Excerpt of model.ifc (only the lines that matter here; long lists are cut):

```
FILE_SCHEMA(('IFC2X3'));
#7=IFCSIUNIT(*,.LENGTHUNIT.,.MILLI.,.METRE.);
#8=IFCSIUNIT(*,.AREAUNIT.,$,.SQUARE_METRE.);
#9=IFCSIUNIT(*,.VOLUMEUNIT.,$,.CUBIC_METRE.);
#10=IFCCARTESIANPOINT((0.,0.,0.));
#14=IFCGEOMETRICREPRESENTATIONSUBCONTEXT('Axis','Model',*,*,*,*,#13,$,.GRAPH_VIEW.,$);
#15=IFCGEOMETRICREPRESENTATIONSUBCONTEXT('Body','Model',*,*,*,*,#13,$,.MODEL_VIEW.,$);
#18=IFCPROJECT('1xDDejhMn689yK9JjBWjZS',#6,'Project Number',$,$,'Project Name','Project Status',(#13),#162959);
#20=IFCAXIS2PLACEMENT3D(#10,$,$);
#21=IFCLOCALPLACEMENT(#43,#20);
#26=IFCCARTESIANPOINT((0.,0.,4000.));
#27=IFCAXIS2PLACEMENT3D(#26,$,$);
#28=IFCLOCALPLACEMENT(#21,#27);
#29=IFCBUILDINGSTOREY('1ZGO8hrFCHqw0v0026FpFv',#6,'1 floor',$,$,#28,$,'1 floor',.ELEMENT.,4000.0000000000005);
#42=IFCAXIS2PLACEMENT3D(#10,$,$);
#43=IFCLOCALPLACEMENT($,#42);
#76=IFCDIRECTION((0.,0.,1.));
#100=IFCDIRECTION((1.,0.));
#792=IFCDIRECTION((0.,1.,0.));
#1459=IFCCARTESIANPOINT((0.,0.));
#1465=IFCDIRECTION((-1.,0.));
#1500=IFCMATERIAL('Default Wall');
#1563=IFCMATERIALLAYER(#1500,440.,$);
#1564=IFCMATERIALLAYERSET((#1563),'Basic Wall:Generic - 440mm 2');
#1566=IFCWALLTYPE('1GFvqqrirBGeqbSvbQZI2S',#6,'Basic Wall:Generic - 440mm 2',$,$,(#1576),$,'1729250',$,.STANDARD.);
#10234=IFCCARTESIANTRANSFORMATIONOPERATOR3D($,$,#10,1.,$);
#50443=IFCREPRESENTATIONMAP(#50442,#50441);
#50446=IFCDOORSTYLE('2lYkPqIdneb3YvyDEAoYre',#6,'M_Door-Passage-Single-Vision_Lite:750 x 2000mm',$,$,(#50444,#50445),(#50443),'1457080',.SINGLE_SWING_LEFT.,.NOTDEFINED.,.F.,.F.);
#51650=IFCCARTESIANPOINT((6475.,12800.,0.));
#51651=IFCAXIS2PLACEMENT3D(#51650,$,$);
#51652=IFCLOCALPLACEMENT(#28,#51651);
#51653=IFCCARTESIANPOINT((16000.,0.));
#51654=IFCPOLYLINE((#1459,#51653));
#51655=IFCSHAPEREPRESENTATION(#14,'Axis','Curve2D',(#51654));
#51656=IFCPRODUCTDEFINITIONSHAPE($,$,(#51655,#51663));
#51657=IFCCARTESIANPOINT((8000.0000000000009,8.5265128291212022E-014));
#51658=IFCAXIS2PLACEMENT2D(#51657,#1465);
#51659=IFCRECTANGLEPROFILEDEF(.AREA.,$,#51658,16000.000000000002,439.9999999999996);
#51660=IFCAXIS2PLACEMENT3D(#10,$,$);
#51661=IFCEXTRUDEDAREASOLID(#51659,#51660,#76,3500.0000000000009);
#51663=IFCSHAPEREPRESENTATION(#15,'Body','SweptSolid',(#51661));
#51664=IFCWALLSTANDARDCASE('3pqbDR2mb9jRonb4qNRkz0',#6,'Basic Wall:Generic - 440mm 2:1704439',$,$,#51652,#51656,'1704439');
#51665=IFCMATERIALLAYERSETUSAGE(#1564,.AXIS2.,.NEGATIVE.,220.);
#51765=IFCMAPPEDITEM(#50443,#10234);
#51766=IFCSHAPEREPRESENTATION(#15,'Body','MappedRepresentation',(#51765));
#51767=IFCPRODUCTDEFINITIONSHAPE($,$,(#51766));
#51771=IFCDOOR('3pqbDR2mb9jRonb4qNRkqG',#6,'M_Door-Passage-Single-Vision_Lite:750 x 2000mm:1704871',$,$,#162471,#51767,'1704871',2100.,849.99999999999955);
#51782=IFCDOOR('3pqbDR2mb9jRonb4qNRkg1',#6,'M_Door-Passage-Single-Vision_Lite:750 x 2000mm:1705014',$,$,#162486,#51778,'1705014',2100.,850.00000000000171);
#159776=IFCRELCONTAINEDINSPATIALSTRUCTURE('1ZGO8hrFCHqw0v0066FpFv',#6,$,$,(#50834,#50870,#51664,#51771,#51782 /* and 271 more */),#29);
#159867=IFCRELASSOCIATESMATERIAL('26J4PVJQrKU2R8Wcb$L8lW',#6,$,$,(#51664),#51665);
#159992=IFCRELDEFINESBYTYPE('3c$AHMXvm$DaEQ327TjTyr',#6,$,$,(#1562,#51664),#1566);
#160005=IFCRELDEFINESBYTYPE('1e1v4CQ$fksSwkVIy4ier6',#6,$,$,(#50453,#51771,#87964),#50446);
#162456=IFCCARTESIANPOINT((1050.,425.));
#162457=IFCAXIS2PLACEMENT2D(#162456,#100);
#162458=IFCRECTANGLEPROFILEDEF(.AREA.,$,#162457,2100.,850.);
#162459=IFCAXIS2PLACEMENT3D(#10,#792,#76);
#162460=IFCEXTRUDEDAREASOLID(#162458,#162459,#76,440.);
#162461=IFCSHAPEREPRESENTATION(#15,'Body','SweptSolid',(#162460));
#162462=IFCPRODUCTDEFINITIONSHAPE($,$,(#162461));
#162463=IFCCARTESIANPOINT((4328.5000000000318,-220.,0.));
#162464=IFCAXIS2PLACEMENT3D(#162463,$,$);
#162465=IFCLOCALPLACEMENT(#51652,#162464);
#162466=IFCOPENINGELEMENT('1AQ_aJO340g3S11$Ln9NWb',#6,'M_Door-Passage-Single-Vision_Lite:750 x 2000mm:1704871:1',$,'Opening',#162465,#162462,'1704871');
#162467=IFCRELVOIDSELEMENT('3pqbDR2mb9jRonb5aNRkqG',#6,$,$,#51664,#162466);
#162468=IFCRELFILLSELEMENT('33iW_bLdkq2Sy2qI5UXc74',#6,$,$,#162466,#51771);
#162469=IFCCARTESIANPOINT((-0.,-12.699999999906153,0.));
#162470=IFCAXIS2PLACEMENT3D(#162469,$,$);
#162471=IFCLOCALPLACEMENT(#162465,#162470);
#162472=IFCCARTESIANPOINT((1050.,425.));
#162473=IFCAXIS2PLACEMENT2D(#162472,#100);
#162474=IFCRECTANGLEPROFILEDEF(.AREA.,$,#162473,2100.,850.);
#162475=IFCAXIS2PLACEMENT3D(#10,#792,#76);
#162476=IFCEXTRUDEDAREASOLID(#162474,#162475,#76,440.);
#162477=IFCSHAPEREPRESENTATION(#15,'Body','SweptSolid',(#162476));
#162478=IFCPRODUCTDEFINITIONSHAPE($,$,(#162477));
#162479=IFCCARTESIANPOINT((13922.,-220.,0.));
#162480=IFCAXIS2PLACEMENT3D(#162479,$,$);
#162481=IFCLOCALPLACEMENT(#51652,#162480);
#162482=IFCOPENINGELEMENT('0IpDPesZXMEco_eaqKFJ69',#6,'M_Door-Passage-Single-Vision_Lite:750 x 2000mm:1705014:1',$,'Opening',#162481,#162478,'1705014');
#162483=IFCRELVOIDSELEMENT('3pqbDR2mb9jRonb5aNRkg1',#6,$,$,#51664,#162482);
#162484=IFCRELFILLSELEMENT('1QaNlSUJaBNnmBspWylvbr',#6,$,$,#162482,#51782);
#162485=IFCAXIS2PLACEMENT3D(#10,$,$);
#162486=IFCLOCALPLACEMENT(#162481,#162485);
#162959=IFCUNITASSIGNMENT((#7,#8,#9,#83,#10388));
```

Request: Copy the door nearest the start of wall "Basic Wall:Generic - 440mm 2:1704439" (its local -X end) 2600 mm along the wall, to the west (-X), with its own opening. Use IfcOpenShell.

```python
import ifcopenshell
import ifcopenshell.api.feature
import ifcopenshell.api.geometry
import ifcopenshell.api.root
import ifcopenshell.geom
import ifcopenshell.util.element
import ifcopenshell.util.placement
import ifcopenshell.util.shape
import ifcopenshell.util.unit

model = ifcopenshell.open("model.ifc")
unit_scale = ifcopenshell.util.unit.calculate_unit_scale(model)
settings = ifcopenshell.geom.settings()


def volume(element):
    """Net volume in cubic metres, openings subtracted."""
    shape = ifcopenshell.geom.create_shape(settings, element)
    return ifcopenshell.util.shape.get_volume(shape.geometry)


def reuse_history(source, copy):
    """copy_class also copies each property set's owner history, people and application; keep the originals."""
    for rel in copy.IsDefinedBy:
        if rel.is_a("IfcRelDefinesByProperties") and (history := rel.RelatingPropertyDefinition.OwnerHistory):
            rel.RelatingPropertyDefinition.OwnerHistory = source.OwnerHistory
            ifcopenshell.util.element.remove_deep2(model, history)


door = model.by_id(51771)
opening = door.FillsVoids[0].RelatingOpeningElement
wall = opening.VoidsElements[0].RelatingBuildingElement
before = volume(wall)
shift = ifcopenshell.util.placement.get_local_placement(wall.ObjectPlacement)[:3, 0] * -2.6 / unit_scale

# copy_class copies the void relationship, type, container and properties, but no geometry.
new_opening = ifcopenshell.api.root.copy_class(model, product=opening)
new_opening.Representation = ifcopenshell.util.element.copy_deep(
    model, opening.Representation, exclude=["IfcGeometricRepresentationContext", "IfcRepresentationMap"]
)
new_opening.Name = "M_Door-Passage-Single-Vision_Lite:750 x 2000mm"
new_opening.Tag = None
new_door = ifcopenshell.api.root.copy_class(model, product=door)
new_door.Representation = ifcopenshell.util.element.copy_deep(
    model, door.Representation, exclude=["IfcGeometricRepresentationContext", "IfcRepresentationMap"]
)
new_door.Name = "M_Door-Passage-Single-Vision_Lite:750 x 2000mm"
new_door.Tag = None
reuse_history(door, new_door)
fills = ifcopenshell.api.feature.add_filling(model, opening=new_opening, element=new_door)
fills.OwnerHistory = new_door.OwnerHistory  # required in IFC2X3

for old, new in ((opening, new_opening), (door, new_door)):
    matrix = ifcopenshell.util.placement.get_local_placement(old.ObjectPlacement)
    matrix[:3, 3] += shift
    ifcopenshell.api.geometry.edit_object_placement(model, product=new, matrix=matrix, is_si=False)

after = volume(wall)

print(f"wall volume {before:.3f} -> {after:.3f} m3")

model.write("model-out.ifc")
```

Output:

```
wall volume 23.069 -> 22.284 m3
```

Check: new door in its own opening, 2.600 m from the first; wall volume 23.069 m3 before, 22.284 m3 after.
